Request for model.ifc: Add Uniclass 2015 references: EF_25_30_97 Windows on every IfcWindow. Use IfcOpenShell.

First a look at what the model holds.

```python
import ifcopenshell

model = ifcopenshell.open("model.ifc")
print(model.schema)
print("classifications:", [c.Name for c in model.by_type("IfcClassification")])
for ifc_class in ("IfcDoor", "IfcRoof", "IfcStair", "IfcWall", "IfcWindow"):
    print(ifc_class, len(model.by_type(ifc_class)))
```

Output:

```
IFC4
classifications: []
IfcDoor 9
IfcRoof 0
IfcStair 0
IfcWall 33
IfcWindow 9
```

```python
import ifcopenshell
import ifcopenshell.api.classification

model = ifcopenshell.open("model.ifc")

system = ifcopenshell.api.classification.add_classification(model, classification="Uniclass 2015")

codes = {
    "IfcWindow": ("EF_25_30_97", "Windows"),
}
for ifc_class, (code, name) in codes.items():
    products = model.by_type(ifc_class)
    ifcopenshell.api.classification.add_reference(
        model, products=products, classification=system, identification=code, name=name
    )
    print(code, len(products))

model.write("model_updated.ifc")
```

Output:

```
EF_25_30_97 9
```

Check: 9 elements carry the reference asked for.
